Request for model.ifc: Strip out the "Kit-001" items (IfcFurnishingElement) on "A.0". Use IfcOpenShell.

First a look at what the model holds.

```python
import ifcopenshell
import ifcopenshell.util.element

model = ifcopenshell.open("model.ifc")
print(model.schema)
storey = next(s for s in model.by_type("IfcBuildingStorey") if s.Name == "A.0")
furniture = [e for e in ifcopenshell.util.element.get_decomposition(storey) if e.is_a("IfcFurnishingElement")]
seen = {}
for e in furniture:
    element_type = ifcopenshell.util.element.get_type(e)
    name = element_type.Name if element_type not in (None, e) else None
    seen[name] = seen.get(name, 0) + 1
for name, count in sorted(seen.items(), key=str):
    print(count, "x", name)
```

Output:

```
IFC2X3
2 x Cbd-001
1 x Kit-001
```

```python
import ifcopenshell
import ifcopenshell.api.root
import ifcopenshell.util.element

model = ifcopenshell.open("model.ifc")

storey = next(s for s in model.by_type("IfcBuildingStorey") if s.Name == "A.0")
furniture = [e for e in ifcopenshell.util.element.get_decomposition(storey) if e.is_a("IfcFurnishingElement")]
targets = [e for e in furniture if (t := ifcopenshell.util.element.get_type(e)) not in (None, e) and t.Name == "Kit-001"]

for e in targets:
    ifcopenshell.api.root.remove_product(model, product=e)
print(len(targets), "removed")

model.write("model_v2.ifc")
```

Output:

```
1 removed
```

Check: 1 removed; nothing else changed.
